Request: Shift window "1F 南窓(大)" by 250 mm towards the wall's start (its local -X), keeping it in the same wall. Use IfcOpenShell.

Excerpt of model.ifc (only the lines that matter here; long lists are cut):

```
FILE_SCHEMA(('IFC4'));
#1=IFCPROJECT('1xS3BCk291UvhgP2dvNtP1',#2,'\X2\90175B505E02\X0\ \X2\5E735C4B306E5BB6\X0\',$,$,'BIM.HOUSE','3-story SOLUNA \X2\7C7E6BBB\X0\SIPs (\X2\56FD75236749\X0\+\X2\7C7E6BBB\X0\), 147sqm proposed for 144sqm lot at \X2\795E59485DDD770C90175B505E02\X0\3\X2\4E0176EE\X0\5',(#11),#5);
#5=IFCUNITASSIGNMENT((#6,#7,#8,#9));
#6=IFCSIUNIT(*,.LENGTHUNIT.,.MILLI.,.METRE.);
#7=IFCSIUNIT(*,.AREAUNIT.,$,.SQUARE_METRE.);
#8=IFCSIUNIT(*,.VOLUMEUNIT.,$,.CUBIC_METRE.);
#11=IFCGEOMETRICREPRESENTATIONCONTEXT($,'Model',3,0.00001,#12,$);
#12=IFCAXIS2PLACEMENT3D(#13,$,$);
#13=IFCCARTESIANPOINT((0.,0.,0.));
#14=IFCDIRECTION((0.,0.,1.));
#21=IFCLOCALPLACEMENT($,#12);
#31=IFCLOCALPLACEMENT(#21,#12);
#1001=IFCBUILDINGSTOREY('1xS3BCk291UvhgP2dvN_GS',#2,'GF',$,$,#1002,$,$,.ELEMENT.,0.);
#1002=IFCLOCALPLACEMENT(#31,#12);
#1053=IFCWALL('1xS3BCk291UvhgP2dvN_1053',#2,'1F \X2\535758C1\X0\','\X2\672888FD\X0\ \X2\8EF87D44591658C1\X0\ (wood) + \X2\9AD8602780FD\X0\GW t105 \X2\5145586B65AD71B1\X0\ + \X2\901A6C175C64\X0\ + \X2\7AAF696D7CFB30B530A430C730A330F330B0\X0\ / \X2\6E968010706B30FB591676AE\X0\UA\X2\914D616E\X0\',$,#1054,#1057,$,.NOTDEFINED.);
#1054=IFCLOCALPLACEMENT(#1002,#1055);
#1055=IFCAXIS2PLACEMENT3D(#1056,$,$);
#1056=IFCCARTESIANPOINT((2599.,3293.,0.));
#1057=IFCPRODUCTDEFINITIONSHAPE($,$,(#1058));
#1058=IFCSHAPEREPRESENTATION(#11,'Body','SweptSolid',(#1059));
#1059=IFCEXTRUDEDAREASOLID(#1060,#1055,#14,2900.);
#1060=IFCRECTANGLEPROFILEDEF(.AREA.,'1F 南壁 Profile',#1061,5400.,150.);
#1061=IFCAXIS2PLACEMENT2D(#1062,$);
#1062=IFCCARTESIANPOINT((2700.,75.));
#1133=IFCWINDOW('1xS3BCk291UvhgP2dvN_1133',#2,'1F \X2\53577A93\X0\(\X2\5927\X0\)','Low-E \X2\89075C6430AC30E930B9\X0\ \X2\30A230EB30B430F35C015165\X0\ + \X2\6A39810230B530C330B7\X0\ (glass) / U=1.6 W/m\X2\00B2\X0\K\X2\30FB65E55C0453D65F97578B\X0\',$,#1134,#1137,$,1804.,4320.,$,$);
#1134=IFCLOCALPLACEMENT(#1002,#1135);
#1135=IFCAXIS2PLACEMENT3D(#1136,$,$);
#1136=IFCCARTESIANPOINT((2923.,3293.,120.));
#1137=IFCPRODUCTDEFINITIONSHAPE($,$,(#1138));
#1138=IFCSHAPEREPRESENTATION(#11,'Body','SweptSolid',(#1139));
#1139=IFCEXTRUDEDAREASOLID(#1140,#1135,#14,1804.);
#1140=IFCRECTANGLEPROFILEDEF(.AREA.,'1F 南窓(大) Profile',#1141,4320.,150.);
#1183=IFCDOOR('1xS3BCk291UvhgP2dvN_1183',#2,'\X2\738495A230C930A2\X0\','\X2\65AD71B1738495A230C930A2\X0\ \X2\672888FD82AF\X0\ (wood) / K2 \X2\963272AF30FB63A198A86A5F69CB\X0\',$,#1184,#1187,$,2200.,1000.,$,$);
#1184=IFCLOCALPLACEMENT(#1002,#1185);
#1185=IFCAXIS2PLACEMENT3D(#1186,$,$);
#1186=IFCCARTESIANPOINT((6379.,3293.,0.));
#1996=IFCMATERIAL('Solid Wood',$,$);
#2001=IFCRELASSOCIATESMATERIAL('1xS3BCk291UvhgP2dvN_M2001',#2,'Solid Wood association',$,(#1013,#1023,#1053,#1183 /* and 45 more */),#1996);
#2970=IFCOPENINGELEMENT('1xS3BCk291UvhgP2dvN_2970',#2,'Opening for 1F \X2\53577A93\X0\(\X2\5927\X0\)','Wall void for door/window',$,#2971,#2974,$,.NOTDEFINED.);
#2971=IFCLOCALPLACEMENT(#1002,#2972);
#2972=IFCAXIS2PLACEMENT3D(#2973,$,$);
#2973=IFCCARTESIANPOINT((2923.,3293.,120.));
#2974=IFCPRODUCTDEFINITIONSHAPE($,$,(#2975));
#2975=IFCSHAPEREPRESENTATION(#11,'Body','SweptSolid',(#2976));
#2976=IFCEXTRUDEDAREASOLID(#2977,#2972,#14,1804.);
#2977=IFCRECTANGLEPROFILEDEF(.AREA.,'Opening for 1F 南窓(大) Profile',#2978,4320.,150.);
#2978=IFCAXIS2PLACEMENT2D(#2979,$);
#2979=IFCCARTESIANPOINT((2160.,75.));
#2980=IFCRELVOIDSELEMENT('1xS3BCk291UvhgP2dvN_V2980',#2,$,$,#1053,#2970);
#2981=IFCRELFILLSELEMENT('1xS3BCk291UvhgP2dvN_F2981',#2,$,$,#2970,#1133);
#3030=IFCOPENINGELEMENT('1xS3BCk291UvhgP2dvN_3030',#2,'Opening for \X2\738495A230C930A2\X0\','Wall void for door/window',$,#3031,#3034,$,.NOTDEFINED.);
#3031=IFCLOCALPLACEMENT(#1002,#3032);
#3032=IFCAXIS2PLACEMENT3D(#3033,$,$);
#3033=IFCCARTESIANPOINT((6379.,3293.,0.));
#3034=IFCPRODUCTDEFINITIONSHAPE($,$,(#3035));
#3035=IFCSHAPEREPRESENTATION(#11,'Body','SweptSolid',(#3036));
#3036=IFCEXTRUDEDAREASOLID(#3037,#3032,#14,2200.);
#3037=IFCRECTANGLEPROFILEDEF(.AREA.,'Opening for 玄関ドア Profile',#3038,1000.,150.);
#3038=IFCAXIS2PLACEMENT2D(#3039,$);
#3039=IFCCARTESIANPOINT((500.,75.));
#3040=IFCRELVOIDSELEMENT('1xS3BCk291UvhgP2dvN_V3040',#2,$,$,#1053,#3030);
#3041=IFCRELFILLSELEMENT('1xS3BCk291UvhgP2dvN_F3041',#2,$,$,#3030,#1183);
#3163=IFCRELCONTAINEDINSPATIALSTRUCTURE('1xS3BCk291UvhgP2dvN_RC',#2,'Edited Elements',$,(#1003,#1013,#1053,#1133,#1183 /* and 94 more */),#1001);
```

```python
import ifcopenshell
import ifcopenshell.api.geometry
import ifcopenshell.util.placement
import ifcopenshell.util.unit

model = ifcopenshell.open("model.ifc")
unit_scale = ifcopenshell.util.unit.calculate_unit_scale(model)

window = model.by_guid("1xS3BCk291UvhgP2dvN_1133")
opening = window.FillsVoids[0].RelatingOpeningElement
wall = opening.VoidsElements[0].RelatingBuildingElement

wall_matrix = ifcopenshell.util.placement.get_local_placement(wall.ObjectPlacement)
shift = wall_matrix[:3, 0] * -0.25 / unit_scale
before = ifcopenshell.util.placement.get_local_placement(window.ObjectPlacement)[:3, 3].copy()

# The window is not placed relative to its opening, so move both.
for product in (opening, window):
    matrix = ifcopenshell.util.placement.get_local_placement(product.ObjectPlacement)
    matrix[:3, 3] += shift
    ifcopenshell.api.geometry.edit_object_placement(model, product=product, matrix=matrix, is_si=False)

after = ifcopenshell.util.placement.get_local_placement(window.ObjectPlacement)[:3, 3]
print("window moved by", (after - before).round(3) + 0.0)

model.write("model-out.ifc")
```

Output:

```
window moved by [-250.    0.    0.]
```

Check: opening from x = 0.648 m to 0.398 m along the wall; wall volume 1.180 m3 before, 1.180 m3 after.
